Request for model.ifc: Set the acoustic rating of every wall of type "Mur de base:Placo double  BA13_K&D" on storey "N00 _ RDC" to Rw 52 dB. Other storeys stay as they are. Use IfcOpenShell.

First a look at what the model holds.

```python
import ifcopenshell
import ifcopenshell.util.element

model = ifcopenshell.open("model.ifc")
print(model.schema)
storey = next(s for s in model.by_type("IfcBuildingStorey") if s.Name == "N00 _ RDC")
walls = [e for e in ifcopenshell.util.element.get_decomposition(storey) if e.is_a("IfcWall")]
seen = {}
for e in walls:
    element_type = ifcopenshell.util.element.get_type(e)
    key = (element_type.Name if element_type != e and element_type else None, ifcopenshell.util.element.get_pset(e, "Pset_WallCommon", "AcousticRating"))
    seen[key] = seen.get(key, 0) + 1
for (name, value), count in sorted(seen.items(), key=str):
    print(count, "x", name, "|", value)
```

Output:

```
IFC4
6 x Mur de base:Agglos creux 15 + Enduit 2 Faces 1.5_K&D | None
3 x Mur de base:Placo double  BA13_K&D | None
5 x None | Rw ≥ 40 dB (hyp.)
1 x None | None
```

```python
import ifcopenshell
import ifcopenshell.api.pset
import ifcopenshell.util.element

model = ifcopenshell.open("model.ifc")

storey = next(s for s in model.by_type("IfcBuildingStorey") if s.Name == "N00 _ RDC")
walls = [e for e in ifcopenshell.util.element.get_decomposition(storey) if e.is_a("IfcWall")]

count = 0
for e in walls:
    element_type = ifcopenshell.util.element.get_type(e)
    if element_type in (None, e) or element_type.Name != "Mur de base:Placo double  BA13_K&D":
        continue
    # add_pset returns the element's existing set when there is one.
    pset = ifcopenshell.api.pset.add_pset(model, product=e, name="Pset_WallCommon")
    ifcopenshell.api.pset.edit_pset(model, pset=pset, properties={"AcousticRating": "Rw 52 dB"})
    count += 1

print(count, "walls updated")

model.write("model_updated.ifc")
```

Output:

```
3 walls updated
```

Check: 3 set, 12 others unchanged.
